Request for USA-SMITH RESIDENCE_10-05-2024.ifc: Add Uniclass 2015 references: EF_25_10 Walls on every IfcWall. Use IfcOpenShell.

First a look at what the model holds.

```python
import ifcopenshell

model = ifcopenshell.open("USA-SMITH RESIDENCE_10-05-2024.ifc")
print(model.schema)
print("classifications:", [c.Name for c in model.by_type("IfcClassification")])
for ifc_class in ("IfcDoor", "IfcRoof", "IfcStair", "IfcWall", "IfcWindow"):
    print(ifc_class, len(model.by_type(ifc_class)))
```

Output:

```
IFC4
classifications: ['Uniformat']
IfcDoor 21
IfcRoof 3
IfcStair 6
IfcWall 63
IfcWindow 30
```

```python
import ifcopenshell
import ifcopenshell.api.classification

model = ifcopenshell.open("USA-SMITH RESIDENCE_10-05-2024.ifc")

system = ifcopenshell.api.classification.add_classification(model, classification="Uniclass 2015")

codes = {
    "IfcWall": ("EF_25_10", "Walls"),
}
for ifc_class, (code, name) in codes.items():
    products = model.by_type(ifc_class)
    ifcopenshell.api.classification.add_reference(
        model, products=products, classification=system, identification=code, name=name
    )
    print(code, len(products))

model.write("USA-SMITH RESIDENCE_10-05-2024_v2.ifc")
```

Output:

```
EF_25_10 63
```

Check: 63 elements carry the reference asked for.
